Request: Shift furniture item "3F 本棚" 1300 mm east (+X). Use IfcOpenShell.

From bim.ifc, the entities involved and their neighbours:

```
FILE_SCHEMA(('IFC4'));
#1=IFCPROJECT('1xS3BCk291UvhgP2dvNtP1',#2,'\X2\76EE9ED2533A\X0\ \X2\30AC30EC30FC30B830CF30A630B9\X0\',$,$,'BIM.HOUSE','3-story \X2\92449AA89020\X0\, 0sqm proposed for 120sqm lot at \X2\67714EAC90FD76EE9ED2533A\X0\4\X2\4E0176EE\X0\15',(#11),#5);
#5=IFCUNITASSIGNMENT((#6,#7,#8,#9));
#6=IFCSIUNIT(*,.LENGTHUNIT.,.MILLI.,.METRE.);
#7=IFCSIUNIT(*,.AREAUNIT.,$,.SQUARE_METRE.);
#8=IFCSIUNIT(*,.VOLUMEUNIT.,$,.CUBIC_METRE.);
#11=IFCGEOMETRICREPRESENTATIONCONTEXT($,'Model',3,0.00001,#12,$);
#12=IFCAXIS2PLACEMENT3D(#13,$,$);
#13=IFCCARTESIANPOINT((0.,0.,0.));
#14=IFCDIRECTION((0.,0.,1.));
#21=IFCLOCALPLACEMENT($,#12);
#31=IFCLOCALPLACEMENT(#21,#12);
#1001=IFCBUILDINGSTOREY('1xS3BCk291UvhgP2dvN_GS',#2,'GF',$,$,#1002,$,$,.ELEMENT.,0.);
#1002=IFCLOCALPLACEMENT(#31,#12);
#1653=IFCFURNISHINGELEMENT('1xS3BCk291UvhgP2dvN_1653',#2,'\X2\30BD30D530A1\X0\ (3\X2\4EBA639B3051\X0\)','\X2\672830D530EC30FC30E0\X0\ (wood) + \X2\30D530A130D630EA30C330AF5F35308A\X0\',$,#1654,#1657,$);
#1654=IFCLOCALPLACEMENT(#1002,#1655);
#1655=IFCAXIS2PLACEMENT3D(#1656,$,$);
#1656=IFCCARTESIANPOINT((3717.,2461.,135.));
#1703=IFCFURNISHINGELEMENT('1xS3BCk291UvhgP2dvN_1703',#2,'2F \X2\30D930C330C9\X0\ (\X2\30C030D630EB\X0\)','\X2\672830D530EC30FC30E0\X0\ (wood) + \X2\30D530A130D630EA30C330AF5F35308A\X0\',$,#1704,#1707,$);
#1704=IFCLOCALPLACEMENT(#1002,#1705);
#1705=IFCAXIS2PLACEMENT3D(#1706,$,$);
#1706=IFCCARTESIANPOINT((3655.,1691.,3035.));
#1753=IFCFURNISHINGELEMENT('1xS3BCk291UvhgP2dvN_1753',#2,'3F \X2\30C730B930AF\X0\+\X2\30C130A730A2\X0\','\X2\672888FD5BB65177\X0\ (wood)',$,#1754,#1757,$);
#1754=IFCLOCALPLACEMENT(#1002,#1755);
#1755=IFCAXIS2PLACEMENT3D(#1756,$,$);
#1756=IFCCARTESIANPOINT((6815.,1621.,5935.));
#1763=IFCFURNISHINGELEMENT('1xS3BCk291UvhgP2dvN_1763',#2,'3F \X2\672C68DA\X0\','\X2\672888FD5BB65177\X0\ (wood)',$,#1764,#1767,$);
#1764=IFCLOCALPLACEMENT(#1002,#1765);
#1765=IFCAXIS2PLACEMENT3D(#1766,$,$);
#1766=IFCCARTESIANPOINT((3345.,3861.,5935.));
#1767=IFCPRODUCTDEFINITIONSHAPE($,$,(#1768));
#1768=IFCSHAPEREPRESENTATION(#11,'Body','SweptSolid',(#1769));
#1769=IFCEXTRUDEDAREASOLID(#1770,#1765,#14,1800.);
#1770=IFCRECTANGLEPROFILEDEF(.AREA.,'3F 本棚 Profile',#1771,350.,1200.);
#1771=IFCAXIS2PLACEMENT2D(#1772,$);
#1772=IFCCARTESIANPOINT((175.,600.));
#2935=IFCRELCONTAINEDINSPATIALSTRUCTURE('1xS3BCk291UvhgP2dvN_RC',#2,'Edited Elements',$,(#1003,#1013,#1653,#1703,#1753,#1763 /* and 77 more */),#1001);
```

```python
import ifcopenshell
import ifcopenshell.api.geometry
import ifcopenshell.util.placement
import ifcopenshell.util.unit

model = ifcopenshell.open("bim.ifc")
unit_scale = ifcopenshell.util.unit.calculate_unit_scale(model)

item = model.by_guid("1xS3BCk291UvhgP2dvN_1763")
matrix = ifcopenshell.util.placement.get_local_placement(item.ObjectPlacement)
matrix[0, 3] += 1.3 / unit_scale
ifcopenshell.api.geometry.edit_object_placement(model, product=item, matrix=matrix, is_si=False)

print(ifcopenshell.util.placement.get_local_placement(item.ObjectPlacement).round(3) + 0.0)

model.write("bim_rev.ifc")
```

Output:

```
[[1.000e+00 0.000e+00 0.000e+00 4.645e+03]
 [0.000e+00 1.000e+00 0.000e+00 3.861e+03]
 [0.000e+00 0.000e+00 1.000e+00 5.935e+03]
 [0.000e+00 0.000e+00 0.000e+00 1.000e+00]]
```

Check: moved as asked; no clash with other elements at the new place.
